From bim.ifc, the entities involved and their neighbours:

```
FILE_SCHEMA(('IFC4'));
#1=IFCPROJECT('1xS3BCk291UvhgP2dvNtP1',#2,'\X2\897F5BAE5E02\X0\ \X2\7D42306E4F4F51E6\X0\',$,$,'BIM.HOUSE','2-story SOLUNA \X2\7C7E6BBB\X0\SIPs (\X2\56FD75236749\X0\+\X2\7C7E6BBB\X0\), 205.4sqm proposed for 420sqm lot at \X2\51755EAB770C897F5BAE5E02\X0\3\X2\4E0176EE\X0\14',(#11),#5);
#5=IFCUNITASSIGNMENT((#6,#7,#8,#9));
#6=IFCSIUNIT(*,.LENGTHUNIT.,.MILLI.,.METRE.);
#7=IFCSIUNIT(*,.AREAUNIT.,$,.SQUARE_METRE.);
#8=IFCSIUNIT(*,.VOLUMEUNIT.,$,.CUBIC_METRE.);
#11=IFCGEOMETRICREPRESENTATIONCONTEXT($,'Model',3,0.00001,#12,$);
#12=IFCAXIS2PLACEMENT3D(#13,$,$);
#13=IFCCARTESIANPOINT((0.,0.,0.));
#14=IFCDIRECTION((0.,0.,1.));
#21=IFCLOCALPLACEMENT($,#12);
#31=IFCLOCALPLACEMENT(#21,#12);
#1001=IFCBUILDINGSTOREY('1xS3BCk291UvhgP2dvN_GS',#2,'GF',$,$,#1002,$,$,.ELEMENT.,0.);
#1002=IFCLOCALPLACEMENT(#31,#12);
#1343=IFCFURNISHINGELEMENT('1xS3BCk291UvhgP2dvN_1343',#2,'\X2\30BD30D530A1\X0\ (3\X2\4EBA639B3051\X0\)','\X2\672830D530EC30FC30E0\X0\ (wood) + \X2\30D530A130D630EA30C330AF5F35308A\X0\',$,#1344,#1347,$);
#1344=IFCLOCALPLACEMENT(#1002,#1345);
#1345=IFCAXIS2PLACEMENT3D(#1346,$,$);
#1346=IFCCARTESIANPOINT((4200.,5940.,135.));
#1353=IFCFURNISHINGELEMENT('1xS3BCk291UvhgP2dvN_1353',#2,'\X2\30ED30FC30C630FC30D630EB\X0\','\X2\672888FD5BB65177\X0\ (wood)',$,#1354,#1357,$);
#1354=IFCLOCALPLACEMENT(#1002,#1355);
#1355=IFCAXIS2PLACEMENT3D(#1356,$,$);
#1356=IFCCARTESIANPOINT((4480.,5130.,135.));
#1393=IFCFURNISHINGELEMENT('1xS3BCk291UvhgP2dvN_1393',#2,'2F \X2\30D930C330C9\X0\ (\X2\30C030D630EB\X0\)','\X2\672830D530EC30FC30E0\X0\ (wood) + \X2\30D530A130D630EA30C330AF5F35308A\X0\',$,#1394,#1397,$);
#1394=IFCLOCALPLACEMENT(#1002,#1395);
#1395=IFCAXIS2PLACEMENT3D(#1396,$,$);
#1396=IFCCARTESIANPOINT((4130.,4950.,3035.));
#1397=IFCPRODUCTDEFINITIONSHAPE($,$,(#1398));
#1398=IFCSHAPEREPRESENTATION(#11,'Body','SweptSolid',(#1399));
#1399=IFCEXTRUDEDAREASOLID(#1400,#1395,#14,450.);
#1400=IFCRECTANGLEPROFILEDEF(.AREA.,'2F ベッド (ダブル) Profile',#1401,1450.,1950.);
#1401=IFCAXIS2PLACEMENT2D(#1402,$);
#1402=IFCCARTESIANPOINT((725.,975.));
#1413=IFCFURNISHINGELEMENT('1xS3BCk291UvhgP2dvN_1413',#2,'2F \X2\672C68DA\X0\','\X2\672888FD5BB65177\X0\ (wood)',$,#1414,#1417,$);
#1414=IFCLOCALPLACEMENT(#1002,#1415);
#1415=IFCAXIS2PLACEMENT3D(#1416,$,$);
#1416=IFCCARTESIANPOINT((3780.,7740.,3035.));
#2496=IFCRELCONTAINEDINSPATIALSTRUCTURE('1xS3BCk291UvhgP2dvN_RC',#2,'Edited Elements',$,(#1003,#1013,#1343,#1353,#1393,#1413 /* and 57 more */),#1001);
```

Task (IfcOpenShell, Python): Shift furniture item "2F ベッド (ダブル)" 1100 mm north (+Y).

```python
import ifcopenshell
import ifcopenshell.api.geometry
import ifcopenshell.util.placement

model = ifcopenshell.open("bim.ifc")

item = model.by_guid("1xS3BCk291UvhgP2dvN_1393")
matrix = ifcopenshell.util.placement.get_local_placement(item.ObjectPlacement)
matrix[1, 3] += 1100.0
ifcopenshell.api.geometry.edit_object_placement(model, product=item, matrix=matrix, is_si=False)

print(ifcopenshell.util.placement.get_local_placement(item.ObjectPlacement).round(3) + 0.0)

model.write("bim-out.ifc")
```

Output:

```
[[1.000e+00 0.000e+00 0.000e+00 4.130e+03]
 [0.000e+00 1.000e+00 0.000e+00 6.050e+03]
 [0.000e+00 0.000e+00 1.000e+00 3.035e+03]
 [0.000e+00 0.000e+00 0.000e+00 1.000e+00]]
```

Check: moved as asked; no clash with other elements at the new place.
